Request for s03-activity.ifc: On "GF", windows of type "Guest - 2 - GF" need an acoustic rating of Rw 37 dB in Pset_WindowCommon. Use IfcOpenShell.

First a look at what the model holds.

```python
import ifcopenshell
import ifcopenshell.util.element

model = ifcopenshell.open("s03-activity.ifc")
print(model.schema)
storey = next(s for s in model.by_type("IfcBuildingStorey") if s.Name == "GF")
windows = [e for e in ifcopenshell.util.element.get_decomposition(storey) if e.is_a("IfcWindow")]
seen = {}
for e in windows:
    element_type = ifcopenshell.util.element.get_type(e)
    key = (element_type.Name if element_type != e and element_type else None, ifcopenshell.util.element.get_pset(e, "Pset_WindowCommon", "AcousticRating"))
    seen[key] = seen.get(key, 0) + 1
for (name, value), count in sorted(seen.items(), key=str):
    print(count, "x", name, "|", value)
```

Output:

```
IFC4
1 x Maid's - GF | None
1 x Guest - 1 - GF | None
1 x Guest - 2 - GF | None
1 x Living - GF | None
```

```python
import ifcopenshell
import ifcopenshell.api.pset
import ifcopenshell.util.element

model = ifcopenshell.open("s03-activity.ifc")

storey = next(s for s in model.by_type("IfcBuildingStorey") if s.Name == "GF")
windows = [e for e in ifcopenshell.util.element.get_decomposition(storey) if e.is_a("IfcWindow")]

count = 0
for e in windows:
    element_type = ifcopenshell.util.element.get_type(e)
    if element_type in (None, e) or element_type.Name != "Guest - 2 - GF":
        continue
    # add_pset returns the element's existing set when there is one.
    pset = ifcopenshell.api.pset.add_pset(model, product=e, name="Pset_WindowCommon")
    ifcopenshell.api.pset.edit_pset(model, pset=pset, properties={"AcousticRating": "Rw 37 dB"})
    count += 1

print(count, "windows updated")

model.write("s03-activity-out.ifc")
```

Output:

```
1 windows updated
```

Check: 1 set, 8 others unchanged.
